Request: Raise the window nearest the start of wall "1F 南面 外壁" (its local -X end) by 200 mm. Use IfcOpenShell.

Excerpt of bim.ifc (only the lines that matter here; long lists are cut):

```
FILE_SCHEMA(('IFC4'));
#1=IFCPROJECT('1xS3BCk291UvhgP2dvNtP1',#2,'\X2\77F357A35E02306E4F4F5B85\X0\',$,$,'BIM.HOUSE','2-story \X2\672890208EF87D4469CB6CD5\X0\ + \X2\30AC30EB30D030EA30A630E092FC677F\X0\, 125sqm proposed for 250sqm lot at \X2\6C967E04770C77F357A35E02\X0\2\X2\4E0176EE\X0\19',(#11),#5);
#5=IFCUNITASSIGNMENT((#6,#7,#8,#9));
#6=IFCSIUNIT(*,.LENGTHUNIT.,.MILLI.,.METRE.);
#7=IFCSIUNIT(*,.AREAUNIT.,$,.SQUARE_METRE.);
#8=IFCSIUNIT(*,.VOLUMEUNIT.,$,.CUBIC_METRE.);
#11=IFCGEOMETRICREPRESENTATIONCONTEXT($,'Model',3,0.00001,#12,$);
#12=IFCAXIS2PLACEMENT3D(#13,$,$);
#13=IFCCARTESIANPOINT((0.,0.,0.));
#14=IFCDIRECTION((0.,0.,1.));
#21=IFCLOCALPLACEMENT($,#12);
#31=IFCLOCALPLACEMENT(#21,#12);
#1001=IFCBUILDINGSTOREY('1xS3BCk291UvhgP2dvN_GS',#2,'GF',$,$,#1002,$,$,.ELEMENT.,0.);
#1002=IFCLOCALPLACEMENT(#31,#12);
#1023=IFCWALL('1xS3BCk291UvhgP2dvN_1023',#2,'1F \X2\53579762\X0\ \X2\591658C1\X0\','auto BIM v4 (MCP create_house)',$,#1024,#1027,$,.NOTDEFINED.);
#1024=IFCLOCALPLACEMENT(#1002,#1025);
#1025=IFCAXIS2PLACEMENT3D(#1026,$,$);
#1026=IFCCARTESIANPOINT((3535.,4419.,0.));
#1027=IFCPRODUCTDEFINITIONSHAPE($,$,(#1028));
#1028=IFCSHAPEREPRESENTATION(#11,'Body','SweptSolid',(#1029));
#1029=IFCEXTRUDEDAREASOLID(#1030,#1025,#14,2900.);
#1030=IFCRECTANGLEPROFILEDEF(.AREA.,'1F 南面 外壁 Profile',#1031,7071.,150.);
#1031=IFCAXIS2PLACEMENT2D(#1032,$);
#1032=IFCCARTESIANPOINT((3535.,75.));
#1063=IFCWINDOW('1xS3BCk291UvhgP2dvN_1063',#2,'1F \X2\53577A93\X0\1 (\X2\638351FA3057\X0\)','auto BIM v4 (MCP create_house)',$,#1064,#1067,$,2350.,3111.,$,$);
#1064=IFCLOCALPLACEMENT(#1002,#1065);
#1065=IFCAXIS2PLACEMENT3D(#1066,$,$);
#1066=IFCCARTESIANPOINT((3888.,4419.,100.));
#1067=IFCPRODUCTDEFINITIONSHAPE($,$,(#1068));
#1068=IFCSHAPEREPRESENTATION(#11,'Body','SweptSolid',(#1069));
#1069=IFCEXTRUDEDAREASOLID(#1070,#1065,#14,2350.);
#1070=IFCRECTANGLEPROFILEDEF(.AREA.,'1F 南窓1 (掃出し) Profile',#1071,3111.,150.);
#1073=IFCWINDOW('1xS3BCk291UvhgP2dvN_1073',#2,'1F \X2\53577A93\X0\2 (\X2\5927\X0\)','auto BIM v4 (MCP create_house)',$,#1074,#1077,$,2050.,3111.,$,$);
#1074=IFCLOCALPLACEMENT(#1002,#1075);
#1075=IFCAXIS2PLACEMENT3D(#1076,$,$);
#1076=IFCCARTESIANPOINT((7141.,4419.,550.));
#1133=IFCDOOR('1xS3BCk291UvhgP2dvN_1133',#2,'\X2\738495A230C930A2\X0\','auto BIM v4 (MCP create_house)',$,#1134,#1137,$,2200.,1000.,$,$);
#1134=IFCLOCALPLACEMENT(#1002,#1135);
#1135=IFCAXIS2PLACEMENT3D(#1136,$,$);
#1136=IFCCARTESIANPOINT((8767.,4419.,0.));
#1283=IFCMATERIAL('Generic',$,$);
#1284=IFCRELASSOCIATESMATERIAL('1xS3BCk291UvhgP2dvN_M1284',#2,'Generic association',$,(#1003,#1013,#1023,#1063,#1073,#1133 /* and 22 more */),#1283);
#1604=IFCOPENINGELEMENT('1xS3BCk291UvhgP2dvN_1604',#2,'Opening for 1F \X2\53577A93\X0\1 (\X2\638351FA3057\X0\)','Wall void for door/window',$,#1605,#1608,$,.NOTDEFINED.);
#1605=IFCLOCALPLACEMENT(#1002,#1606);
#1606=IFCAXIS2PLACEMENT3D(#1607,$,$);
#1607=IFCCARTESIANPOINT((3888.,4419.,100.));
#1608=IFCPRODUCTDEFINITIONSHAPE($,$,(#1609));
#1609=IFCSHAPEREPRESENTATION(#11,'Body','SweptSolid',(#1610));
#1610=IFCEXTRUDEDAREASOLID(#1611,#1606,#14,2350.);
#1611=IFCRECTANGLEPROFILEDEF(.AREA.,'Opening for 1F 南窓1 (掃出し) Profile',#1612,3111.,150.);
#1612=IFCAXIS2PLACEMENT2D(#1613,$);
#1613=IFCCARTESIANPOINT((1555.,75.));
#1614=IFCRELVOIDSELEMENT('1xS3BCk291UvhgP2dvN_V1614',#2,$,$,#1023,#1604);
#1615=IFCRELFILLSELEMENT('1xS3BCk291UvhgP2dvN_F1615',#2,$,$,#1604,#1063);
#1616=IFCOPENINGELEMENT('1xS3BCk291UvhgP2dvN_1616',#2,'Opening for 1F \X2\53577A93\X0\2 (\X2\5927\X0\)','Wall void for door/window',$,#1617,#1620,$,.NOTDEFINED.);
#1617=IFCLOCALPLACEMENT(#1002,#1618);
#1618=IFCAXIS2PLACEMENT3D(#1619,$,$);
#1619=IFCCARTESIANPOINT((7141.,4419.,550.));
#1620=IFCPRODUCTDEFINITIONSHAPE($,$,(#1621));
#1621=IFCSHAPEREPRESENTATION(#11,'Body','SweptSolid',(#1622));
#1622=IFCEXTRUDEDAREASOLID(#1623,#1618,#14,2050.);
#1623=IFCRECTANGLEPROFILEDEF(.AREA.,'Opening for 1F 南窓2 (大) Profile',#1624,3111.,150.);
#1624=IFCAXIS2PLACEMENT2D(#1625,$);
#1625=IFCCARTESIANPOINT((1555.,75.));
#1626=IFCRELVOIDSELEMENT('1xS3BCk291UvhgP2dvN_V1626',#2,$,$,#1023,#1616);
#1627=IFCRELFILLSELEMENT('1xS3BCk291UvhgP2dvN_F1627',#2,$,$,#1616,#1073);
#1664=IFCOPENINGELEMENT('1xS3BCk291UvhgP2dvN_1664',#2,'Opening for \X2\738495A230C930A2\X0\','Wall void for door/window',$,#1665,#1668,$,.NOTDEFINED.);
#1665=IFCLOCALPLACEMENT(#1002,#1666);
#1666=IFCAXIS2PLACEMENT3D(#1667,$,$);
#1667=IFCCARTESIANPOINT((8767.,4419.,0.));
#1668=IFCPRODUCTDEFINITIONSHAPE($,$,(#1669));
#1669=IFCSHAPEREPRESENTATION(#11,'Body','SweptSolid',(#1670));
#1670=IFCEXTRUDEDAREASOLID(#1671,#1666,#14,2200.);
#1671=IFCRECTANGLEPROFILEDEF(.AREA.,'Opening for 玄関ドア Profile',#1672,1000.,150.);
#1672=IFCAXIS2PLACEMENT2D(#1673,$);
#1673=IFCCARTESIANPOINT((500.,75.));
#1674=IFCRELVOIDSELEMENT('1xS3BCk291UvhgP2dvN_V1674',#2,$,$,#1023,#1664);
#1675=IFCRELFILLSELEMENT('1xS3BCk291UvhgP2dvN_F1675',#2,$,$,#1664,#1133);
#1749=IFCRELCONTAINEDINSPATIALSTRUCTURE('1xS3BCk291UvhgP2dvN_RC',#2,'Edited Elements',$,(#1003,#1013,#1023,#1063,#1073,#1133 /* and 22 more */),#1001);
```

```python
import numpy as np
import ifcopenshell
import ifcopenshell.api.geometry
import ifcopenshell.util.placement
import ifcopenshell.util.unit

model = ifcopenshell.open("bim.ifc")
unit_scale = ifcopenshell.util.unit.calculate_unit_scale(model)

window = model.by_guid("1xS3BCk291UvhgP2dvN_1063")
opening = window.FillsVoids[0].RelatingOpeningElement
dz = 0.2 / unit_scale

shift = np.array([0.0, 0.0, dz])
# The window is not placed relative to its opening, so move both.
for product in (opening, window):
    matrix = ifcopenshell.util.placement.get_local_placement(product.ObjectPlacement)
    matrix[:3, 3] += shift
    ifcopenshell.api.geometry.edit_object_placement(model, product=product, matrix=matrix, is_si=False)

print(f"moved by {dz * unit_scale:+.3f} m")

model.write("bim_edited.ifc")
```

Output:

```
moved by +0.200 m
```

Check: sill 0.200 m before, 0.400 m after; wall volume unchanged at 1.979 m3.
